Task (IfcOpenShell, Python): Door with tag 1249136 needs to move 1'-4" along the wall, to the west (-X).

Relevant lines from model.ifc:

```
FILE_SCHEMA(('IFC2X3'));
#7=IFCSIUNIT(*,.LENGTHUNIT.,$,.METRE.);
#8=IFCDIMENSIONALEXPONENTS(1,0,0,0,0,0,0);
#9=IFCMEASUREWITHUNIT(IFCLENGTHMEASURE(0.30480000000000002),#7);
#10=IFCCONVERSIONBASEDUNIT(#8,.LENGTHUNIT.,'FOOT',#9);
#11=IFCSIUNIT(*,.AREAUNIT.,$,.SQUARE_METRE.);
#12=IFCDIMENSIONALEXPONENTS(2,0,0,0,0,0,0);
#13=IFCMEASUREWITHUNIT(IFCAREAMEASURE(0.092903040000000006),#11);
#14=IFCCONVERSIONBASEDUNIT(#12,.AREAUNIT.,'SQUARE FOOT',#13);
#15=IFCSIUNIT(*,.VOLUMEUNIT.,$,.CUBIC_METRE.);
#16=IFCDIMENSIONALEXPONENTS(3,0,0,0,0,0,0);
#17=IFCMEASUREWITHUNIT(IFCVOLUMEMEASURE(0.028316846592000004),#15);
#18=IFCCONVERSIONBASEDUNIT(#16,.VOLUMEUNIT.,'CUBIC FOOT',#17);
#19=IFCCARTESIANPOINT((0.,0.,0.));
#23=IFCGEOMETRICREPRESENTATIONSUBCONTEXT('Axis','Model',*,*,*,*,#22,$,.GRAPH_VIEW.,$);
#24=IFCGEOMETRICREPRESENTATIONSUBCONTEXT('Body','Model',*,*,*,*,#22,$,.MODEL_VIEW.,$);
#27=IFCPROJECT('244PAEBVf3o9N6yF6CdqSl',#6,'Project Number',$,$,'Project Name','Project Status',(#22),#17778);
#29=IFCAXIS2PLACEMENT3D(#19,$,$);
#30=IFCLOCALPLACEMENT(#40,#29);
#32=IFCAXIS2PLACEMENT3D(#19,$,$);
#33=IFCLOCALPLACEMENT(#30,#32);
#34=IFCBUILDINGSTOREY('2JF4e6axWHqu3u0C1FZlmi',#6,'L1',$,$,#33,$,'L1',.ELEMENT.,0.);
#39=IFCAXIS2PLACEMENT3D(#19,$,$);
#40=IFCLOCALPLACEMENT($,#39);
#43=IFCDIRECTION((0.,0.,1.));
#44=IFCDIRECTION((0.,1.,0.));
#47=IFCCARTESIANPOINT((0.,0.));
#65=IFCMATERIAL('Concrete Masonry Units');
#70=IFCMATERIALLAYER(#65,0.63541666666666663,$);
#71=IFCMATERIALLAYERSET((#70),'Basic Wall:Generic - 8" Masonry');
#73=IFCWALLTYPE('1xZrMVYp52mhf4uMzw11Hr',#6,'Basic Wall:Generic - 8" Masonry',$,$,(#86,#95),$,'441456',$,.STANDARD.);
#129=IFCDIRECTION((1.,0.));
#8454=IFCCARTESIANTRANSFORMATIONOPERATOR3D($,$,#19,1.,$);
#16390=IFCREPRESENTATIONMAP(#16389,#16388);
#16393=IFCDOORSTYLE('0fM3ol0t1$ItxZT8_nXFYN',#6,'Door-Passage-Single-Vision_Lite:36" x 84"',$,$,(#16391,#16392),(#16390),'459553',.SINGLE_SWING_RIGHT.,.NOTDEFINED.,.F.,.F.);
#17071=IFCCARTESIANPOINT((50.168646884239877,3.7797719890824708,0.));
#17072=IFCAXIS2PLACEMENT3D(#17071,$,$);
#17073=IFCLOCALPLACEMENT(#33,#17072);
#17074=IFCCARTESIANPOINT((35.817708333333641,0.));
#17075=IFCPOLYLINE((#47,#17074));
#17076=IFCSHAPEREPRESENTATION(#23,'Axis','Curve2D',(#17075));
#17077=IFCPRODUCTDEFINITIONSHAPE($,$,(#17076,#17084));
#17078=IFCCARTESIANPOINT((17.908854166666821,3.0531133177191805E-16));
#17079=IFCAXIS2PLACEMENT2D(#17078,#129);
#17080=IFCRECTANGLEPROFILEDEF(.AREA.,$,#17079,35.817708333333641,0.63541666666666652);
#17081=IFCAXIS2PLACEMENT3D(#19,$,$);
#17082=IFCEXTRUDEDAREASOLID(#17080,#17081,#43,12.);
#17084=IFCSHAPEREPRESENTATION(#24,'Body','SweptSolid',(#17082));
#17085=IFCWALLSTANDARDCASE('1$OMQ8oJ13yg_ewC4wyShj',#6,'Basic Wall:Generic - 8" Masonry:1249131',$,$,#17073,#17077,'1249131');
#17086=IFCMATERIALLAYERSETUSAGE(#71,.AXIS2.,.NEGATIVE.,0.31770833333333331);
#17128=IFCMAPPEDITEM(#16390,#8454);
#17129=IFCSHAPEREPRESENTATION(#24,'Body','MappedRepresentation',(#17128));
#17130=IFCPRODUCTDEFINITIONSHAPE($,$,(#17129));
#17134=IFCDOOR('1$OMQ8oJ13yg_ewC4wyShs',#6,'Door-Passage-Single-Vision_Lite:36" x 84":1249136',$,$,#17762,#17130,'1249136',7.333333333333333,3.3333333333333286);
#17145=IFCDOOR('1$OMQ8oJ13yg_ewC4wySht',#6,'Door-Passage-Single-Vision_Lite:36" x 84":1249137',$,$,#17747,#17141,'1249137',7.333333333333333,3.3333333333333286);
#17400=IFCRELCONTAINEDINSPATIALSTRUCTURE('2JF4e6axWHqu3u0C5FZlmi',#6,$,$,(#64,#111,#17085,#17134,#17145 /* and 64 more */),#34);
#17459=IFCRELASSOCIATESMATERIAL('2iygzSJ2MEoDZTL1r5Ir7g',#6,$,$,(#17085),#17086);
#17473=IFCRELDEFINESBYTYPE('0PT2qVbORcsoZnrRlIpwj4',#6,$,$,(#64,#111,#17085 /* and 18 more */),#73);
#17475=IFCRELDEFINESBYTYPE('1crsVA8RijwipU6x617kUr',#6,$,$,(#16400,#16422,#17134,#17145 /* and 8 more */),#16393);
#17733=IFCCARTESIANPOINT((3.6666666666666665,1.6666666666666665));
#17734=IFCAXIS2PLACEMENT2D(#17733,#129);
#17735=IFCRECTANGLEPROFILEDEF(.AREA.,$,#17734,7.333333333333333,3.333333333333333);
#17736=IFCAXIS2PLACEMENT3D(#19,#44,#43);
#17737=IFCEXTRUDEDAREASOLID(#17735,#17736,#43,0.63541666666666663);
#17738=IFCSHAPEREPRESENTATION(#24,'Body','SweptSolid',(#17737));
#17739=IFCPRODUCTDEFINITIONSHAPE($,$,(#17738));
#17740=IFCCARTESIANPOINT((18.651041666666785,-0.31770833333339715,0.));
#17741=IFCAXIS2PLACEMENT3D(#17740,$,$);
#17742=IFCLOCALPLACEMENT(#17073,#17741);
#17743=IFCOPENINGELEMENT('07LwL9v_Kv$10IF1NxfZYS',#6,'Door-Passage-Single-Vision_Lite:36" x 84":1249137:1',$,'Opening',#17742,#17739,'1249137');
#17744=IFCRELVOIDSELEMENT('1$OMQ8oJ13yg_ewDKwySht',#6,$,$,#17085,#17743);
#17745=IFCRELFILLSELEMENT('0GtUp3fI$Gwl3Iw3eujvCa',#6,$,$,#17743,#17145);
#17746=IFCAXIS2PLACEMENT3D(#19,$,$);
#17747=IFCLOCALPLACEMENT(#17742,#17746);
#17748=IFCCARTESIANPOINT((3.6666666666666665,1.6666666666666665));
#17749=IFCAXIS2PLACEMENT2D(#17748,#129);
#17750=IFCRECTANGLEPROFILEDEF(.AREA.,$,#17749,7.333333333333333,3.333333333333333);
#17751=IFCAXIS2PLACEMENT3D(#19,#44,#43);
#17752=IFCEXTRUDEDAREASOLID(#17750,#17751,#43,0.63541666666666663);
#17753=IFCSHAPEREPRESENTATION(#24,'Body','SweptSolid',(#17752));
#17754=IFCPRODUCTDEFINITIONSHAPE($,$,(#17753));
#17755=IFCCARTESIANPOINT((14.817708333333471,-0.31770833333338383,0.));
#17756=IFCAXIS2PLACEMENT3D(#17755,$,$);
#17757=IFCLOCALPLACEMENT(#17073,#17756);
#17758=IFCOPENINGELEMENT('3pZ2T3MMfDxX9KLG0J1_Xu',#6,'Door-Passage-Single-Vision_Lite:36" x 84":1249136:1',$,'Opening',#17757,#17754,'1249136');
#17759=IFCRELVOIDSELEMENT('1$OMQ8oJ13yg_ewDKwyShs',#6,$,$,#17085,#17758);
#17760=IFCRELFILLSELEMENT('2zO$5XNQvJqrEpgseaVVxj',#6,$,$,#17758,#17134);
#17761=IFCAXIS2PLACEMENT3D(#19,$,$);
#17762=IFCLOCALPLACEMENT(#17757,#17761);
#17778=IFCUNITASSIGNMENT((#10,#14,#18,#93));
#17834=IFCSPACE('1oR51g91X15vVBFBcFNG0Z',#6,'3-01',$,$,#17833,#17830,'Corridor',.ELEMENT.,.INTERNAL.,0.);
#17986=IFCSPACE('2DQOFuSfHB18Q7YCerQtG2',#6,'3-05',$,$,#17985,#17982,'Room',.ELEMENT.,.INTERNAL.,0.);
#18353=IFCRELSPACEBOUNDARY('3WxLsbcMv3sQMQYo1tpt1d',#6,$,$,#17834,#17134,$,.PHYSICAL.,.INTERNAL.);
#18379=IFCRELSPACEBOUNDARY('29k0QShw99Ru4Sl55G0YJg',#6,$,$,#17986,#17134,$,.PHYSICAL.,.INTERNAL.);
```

```python
import ifcopenshell
import ifcopenshell.api.geometry
import ifcopenshell.util.placement
import ifcopenshell.util.unit

model = ifcopenshell.open("model.ifc")
unit_scale = ifcopenshell.util.unit.calculate_unit_scale(model)

door = model.by_guid("1$OMQ8oJ13yg_ewC4wyShs")
opening = door.FillsVoids[0].RelatingOpeningElement
wall = opening.VoidsElements[0].RelatingBuildingElement

wall_matrix = ifcopenshell.util.placement.get_local_placement(wall.ObjectPlacement)
shift = wall_matrix[:3, 0] * -16 * 0.0254 / unit_scale
before = ifcopenshell.util.placement.get_local_placement(door.ObjectPlacement)[:3, 3].copy()

# The door is placed relative to its opening, so it follows when the opening moves.
matrix = ifcopenshell.util.placement.get_local_placement(opening.ObjectPlacement)
matrix[:3, 3] += shift
ifcopenshell.api.geometry.edit_object_placement(
    model, product=opening, matrix=matrix, is_si=False, should_transform_children=True
)

after = ifcopenshell.util.placement.get_local_placement(door.ObjectPlacement)[:3, 3]
print("door moved by", (after - before).round(3) + 0.0)

model.write("model_edited.ifc")
```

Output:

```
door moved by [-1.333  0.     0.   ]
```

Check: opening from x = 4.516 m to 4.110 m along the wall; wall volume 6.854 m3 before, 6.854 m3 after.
